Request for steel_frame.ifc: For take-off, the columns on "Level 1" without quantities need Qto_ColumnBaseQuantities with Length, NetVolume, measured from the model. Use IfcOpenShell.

First a look at what the model holds.

```python
import ifcopenshell
import ifcopenshell.util.element
import ifcopenshell.util.unit

model = ifcopenshell.open("steel_frame.ifc")
print(model.schema)
for unit_type in ("LENGTHUNIT", "AREAUNIT", "VOLUMEUNIT"):
    print(unit_type, ifcopenshell.util.unit.calculate_unit_scale(model, unit_type))
storey = next(s for s in model.by_type("IfcBuildingStorey") if s.Name == "Level 1")
columns = [e for e in ifcopenshell.util.element.get_decomposition(storey) if e.is_a("IfcColumn")]
for e in sorted(columns, key=lambda e: e.id()):
    print(e.id(), e.is_a(), e.Name, list(ifcopenshell.util.element.get_psets(e, qtos_only=True)), sep=" | ")
```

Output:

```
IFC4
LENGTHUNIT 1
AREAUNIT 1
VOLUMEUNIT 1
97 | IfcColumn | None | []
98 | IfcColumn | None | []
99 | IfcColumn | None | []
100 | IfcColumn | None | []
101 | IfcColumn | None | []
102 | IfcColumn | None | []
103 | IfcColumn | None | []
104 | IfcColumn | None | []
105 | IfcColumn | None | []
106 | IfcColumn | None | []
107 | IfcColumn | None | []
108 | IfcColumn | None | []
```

```python
import ifcopenshell
import ifcopenshell.api.pset
import ifcopenshell.geom
import ifcopenshell.util.element
import ifcopenshell.util.shape
import ifcopenshell.util.unit

model = ifcopenshell.open("steel_frame.ifc")
unit_scale = ifcopenshell.util.unit.calculate_unit_scale(model)
volume_scale = ifcopenshell.util.unit.calculate_unit_scale(model, "VOLUMEUNIT")
settings = ifcopenshell.geom.settings()

storey = next(s for s in model.by_type("IfcBuildingStorey") if s.Name == "Level 1")
columns = [e for e in ifcopenshell.util.element.get_decomposition(storey) if e.is_a("IfcColumn")]

for e in sorted(columns, key=lambda e: e.id()):
    if ifcopenshell.util.element.get_psets(e, qtos_only=True, should_inherit=False):
        continue
    # Geometry comes back in metres, in the element's own axes.
    shape = ifcopenshell.geom.create_shape(settings, e)
    values = {
        "Length": ifcopenshell.util.shape.get_z(shape.geometry) / unit_scale,
        "NetVolume": ifcopenshell.util.shape.get_volume(shape.geometry) / volume_scale,
    }
    qto = ifcopenshell.api.pset.add_qto(model, product=e, name="Qto_ColumnBaseQuantities")
    ifcopenshell.api.pset.edit_qto(model, qto=qto, properties=values)
    print(e.id(), {k: round(v, 3) for k, v in values.items()})

model.write("steel_frame_rev.ifc")
```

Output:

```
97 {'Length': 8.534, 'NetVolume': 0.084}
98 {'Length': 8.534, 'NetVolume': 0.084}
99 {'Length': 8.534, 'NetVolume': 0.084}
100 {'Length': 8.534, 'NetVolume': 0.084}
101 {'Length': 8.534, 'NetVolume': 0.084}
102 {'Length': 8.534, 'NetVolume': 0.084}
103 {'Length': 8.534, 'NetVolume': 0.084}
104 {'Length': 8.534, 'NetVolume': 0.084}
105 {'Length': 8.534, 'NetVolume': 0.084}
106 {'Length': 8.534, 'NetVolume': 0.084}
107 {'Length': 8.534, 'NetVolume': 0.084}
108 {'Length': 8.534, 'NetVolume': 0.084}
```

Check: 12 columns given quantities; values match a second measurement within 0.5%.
